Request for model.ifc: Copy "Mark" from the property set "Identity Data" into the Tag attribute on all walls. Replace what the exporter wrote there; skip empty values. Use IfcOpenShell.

First a look at what the model holds.

```python
import ifcopenshell
import ifcopenshell.util.element

model = ifcopenshell.open("model.ifc")
print(model.schema)
walls = model.by_type("IfcWall")
print(len(walls), "walls")
for e in walls[:8]:
    source = ifcopenshell.util.element.get_pset(e, "Identity Data", "Mark")
    target = e.Tag
    print(e.id(), repr(source), repr(target), sep=" | ")
```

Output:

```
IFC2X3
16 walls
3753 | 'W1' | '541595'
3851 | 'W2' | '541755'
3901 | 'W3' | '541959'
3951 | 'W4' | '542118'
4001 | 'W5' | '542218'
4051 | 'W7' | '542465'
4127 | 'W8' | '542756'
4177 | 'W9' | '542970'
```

```python
import ifcopenshell
import ifcopenshell.util.element

model = ifcopenshell.open("model.ifc")

count = 0
for e in model.by_type("IfcWall"):
    value = ifcopenshell.util.element.get_pset(e, "Identity Data", "Mark")
    current = e.Tag
    if not value or not value.strip() or current == value:
        continue
    e.Tag = value
    count += 1

print(count, "walls updated")

model.write("model_edited.ifc")
```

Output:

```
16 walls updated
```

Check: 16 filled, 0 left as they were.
